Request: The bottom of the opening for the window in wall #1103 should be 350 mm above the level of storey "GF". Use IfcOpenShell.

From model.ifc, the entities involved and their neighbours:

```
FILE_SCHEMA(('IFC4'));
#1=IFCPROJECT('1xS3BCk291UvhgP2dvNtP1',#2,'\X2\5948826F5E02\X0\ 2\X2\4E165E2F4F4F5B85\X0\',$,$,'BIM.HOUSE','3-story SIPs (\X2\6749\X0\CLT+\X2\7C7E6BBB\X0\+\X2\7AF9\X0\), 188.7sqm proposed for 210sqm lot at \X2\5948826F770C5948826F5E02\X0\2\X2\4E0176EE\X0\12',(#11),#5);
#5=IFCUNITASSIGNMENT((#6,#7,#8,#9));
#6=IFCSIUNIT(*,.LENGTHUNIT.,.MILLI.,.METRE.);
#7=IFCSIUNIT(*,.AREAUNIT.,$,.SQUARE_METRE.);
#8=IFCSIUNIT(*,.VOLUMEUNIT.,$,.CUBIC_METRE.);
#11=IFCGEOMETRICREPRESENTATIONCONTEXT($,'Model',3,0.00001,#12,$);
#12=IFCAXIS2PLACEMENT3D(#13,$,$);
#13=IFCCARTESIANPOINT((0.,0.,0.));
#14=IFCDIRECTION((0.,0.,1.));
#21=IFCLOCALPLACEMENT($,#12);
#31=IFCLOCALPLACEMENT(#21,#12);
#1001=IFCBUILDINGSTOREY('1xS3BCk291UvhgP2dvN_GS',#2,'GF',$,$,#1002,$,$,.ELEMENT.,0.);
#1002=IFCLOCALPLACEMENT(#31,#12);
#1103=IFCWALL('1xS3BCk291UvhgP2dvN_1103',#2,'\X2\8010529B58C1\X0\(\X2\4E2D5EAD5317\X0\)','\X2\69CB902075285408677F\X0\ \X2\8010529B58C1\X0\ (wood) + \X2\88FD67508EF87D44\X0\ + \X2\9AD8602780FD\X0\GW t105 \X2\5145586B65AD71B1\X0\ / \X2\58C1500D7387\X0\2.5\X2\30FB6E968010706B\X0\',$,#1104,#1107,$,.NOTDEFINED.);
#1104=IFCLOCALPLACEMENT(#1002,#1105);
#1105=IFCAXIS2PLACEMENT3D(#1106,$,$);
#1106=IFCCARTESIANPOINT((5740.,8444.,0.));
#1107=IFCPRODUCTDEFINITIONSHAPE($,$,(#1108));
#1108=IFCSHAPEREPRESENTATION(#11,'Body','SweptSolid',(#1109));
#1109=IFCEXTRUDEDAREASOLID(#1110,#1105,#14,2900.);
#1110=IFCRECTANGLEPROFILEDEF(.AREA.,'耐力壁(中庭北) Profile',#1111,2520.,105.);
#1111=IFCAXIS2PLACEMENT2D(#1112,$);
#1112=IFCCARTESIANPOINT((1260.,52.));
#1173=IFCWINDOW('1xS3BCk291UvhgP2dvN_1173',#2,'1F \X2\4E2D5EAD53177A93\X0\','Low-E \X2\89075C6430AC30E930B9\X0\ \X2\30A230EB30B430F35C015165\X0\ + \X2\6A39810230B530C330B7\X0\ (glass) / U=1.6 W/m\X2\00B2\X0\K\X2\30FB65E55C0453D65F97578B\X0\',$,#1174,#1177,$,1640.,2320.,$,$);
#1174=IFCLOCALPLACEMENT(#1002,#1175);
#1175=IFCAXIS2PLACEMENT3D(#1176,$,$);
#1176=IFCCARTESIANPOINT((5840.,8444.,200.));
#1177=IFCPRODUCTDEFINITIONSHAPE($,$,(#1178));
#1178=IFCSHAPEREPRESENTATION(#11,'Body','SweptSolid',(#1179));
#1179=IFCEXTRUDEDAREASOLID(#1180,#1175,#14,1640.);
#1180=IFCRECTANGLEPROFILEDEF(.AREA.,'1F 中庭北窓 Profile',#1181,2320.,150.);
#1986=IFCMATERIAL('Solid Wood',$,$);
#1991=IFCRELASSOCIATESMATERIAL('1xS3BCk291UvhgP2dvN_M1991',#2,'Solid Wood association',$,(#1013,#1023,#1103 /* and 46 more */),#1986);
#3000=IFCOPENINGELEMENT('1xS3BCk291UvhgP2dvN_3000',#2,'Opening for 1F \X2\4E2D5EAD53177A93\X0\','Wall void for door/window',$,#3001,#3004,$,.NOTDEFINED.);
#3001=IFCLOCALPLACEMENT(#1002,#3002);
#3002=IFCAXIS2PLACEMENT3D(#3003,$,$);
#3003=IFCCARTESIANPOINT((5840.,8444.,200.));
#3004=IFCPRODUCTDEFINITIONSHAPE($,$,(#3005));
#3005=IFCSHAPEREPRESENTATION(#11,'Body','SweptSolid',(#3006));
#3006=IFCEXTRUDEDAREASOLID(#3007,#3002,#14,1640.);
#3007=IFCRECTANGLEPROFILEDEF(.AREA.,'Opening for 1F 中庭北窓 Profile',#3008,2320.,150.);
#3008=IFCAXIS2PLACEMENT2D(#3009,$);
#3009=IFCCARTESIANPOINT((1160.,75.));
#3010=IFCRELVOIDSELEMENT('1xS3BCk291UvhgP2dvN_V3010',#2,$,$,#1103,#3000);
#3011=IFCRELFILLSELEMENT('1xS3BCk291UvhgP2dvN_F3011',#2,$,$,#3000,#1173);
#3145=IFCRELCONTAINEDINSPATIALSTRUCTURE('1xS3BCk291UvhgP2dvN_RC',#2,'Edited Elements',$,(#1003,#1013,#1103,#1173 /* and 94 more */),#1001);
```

```python
import numpy as np
import ifcopenshell
import ifcopenshell.api.geometry
import ifcopenshell.geom
import ifcopenshell.util.element
import ifcopenshell.util.placement
import ifcopenshell.util.shape
import ifcopenshell.util.unit

model = ifcopenshell.open("model.ifc")
unit_scale = ifcopenshell.util.unit.calculate_unit_scale(model)

window = model.by_id(1173)
opening = window.FillsVoids[0].RelatingOpeningElement
storey = ifcopenshell.util.element.get_container(window, ifc_class="IfcBuildingStorey")
level = ifcopenshell.util.placement.get_local_placement(storey.ObjectPlacement)[2, 3]

# The opening's origin need not be at the sill, so measure its lowest point.
shape = ifcopenshell.geom.create_shape(ifcopenshell.geom.settings(), opening)
bottom = ifcopenshell.util.shape.get_shape_bottom_elevation(shape, shape.geometry) / unit_scale
dz = level + 0.35 / unit_scale - bottom

shift = np.array([0.0, 0.0, dz])
# The window is not placed relative to its opening, so move both.
for product in (opening, window):
    matrix = ifcopenshell.util.placement.get_local_placement(product.ObjectPlacement)
    matrix[:3, 3] += shift
    ifcopenshell.api.geometry.edit_object_placement(model, product=product, matrix=matrix, is_si=False)

print(f"moved by {dz * unit_scale:+.3f} m")

model.write("model-out.ifc")
```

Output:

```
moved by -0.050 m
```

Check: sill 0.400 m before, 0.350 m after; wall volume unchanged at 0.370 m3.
